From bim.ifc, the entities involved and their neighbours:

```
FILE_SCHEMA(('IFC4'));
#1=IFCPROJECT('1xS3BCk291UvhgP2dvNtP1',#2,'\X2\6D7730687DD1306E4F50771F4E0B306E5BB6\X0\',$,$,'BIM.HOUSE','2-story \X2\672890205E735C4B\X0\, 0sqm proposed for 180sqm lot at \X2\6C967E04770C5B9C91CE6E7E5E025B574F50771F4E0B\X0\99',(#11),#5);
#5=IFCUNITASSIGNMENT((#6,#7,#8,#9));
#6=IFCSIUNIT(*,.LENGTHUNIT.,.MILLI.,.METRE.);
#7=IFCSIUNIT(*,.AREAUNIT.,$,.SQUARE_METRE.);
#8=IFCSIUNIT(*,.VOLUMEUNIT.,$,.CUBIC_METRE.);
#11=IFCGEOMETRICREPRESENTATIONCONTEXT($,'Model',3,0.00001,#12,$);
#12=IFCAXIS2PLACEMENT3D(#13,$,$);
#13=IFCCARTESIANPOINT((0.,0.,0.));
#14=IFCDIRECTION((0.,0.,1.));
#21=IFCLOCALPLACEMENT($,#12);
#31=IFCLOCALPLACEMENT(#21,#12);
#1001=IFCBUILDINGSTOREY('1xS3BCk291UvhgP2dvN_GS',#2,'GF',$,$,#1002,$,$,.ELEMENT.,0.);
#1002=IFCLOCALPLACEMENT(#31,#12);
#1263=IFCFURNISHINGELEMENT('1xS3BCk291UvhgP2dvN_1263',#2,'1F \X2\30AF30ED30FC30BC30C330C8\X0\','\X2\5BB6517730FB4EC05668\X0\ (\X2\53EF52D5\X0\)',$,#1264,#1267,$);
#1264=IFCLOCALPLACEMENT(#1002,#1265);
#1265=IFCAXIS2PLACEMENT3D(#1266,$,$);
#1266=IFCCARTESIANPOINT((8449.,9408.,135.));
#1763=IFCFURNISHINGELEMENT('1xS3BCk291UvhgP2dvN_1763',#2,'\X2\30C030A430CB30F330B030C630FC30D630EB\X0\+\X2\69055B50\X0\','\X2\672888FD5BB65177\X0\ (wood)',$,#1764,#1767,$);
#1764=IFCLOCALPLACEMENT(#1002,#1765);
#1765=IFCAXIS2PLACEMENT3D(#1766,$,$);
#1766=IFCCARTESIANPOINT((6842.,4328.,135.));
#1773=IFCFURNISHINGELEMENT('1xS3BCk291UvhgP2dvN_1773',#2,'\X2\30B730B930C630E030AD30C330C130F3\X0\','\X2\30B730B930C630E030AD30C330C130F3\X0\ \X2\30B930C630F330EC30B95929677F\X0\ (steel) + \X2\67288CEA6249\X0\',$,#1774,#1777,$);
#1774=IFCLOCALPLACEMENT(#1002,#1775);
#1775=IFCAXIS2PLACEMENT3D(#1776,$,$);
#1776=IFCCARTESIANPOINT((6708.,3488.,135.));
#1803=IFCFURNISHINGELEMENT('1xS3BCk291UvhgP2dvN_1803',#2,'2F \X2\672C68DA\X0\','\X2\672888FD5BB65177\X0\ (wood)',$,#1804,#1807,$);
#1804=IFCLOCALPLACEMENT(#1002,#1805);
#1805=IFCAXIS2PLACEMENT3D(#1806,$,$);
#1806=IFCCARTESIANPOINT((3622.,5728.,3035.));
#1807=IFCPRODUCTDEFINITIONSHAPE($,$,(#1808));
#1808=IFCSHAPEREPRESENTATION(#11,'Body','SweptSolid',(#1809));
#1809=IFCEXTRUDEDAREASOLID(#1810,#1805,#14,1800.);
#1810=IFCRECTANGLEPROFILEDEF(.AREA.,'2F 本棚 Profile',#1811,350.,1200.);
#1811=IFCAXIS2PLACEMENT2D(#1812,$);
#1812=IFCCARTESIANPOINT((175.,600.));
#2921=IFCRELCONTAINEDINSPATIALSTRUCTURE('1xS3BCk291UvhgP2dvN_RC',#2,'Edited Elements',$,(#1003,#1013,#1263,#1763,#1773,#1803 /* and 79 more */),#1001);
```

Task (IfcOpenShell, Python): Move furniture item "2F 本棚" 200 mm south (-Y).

```python
import ifcopenshell
import ifcopenshell.api.geometry
import ifcopenshell.util.placement

model = ifcopenshell.open("bim.ifc")

item = model.by_guid("1xS3BCk291UvhgP2dvN_1803")
matrix = ifcopenshell.util.placement.get_local_placement(item.ObjectPlacement)
matrix[1, 3] -= 200.0
ifcopenshell.api.geometry.edit_object_placement(model, product=item, matrix=matrix, is_si=False)

print(ifcopenshell.util.placement.get_local_placement(item.ObjectPlacement).round(3) + 0.0)

model.write("bim-out.ifc")
```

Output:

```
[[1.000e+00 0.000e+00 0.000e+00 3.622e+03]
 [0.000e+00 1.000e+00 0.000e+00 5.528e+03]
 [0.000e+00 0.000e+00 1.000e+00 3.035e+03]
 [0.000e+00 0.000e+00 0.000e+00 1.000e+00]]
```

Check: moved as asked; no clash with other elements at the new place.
